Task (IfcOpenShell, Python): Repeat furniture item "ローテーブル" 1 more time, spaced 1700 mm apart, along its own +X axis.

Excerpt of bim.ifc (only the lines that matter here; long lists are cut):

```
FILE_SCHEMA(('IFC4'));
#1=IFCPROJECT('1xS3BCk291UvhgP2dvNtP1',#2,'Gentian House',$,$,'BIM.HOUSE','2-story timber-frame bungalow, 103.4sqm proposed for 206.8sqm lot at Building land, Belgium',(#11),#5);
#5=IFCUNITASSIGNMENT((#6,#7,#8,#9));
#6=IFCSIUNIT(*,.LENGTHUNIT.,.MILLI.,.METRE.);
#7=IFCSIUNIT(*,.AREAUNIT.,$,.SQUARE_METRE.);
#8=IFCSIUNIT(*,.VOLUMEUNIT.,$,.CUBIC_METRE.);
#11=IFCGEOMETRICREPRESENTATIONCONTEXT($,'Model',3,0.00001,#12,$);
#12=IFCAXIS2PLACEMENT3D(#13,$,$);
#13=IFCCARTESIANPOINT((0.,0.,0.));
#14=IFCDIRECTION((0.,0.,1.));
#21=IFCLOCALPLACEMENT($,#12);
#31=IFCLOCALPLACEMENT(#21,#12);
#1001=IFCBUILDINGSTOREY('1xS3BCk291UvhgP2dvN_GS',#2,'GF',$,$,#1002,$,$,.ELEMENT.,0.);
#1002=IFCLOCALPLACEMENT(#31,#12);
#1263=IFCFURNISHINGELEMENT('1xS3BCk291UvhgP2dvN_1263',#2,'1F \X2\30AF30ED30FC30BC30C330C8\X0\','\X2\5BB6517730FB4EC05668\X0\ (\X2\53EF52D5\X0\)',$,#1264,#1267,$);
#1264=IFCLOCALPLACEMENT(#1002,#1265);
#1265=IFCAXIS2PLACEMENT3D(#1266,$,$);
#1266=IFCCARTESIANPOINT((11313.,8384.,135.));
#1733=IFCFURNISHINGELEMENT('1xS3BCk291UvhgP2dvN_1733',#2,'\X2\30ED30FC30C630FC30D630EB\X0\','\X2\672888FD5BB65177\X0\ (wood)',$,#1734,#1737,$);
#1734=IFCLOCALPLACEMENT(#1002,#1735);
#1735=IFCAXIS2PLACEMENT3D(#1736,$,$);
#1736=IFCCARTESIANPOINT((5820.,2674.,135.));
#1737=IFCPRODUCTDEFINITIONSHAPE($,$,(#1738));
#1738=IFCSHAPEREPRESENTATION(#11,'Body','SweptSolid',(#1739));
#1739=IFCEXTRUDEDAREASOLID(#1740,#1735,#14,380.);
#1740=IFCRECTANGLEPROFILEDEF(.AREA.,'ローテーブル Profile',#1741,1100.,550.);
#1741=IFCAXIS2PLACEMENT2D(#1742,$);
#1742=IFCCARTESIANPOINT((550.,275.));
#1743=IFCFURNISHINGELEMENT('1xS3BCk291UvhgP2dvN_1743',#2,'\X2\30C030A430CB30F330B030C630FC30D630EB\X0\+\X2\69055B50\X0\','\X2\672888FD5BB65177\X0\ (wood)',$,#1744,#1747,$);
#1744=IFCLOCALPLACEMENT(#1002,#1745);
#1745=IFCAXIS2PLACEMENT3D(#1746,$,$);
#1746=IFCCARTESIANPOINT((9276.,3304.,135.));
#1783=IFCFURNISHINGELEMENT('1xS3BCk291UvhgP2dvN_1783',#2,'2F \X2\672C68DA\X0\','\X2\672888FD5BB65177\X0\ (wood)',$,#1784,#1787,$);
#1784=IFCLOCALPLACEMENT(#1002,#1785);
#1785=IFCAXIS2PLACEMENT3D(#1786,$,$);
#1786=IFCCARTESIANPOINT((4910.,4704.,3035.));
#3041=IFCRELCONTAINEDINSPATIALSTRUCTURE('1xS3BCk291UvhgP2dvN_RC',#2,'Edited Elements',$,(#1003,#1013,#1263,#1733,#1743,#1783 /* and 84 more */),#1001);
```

```python
import ifcopenshell
import ifcopenshell.api.geometry
import ifcopenshell.api.root
import ifcopenshell.util.element
import ifcopenshell.util.placement
import ifcopenshell.util.unit

model = ifcopenshell.open("bim.ifc")
unit_scale = ifcopenshell.util.unit.calculate_unit_scale(model)


def reuse_history(source, copy):
    """copy_class also copies each property set's owner history, people and application; keep the originals."""
    for rel in copy.IsDefinedBy:
        if rel.is_a("IfcRelDefinesByProperties") and (history := rel.RelatingPropertyDefinition.OwnerHistory):
            rel.RelatingPropertyDefinition.OwnerHistory = source.OwnerHistory
            ifcopenshell.util.element.remove_deep2(model, history)


source = model.by_guid("1xS3BCk291UvhgP2dvN_1733")
base = ifcopenshell.util.placement.get_local_placement(source.ObjectPlacement)
step = base[:3, 0] * 1.7 / unit_scale

for i in range(1, 2):
    copy = ifcopenshell.api.root.copy_class(model, product=source)
    copy.Representation = ifcopenshell.util.element.copy_deep(
        model, source.Representation, exclude=["IfcGeometricRepresentationContext", "IfcRepresentationMap"]
    )
    reuse_history(source, copy)
    matrix = base.copy()
    matrix[:3, 3] += i * step
    print("added at", matrix[:3, 3].round(3) + 0.0)
    ifcopenshell.api.geometry.edit_object_placement(model, product=copy, matrix=matrix, is_si=False)

model.write("bim_rev.ifc")
```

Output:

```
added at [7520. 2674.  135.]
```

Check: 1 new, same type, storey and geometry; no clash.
